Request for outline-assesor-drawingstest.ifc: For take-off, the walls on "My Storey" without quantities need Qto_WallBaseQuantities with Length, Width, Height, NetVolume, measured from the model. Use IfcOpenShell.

First a look at what the model holds.

```python
import ifcopenshell
import ifcopenshell.util.element
import ifcopenshell.util.unit

model = ifcopenshell.open("outline-assesor-drawingstest.ifc")
print(model.schema)
for unit_type in ("LENGTHUNIT", "AREAUNIT", "VOLUMEUNIT"):
    print(unit_type, ifcopenshell.util.unit.calculate_unit_scale(model, unit_type))
storey = next(s for s in model.by_type("IfcBuildingStorey") if s.Name == "My Storey")
walls = [e for e in ifcopenshell.util.element.get_decomposition(storey) if e.is_a("IfcWall")]
for e in sorted(walls, key=lambda e: e.id()):
    print(e.id(), e.is_a(), e.Name, list(ifcopenshell.util.element.get_psets(e, qtos_only=True)), sep=" | ")
```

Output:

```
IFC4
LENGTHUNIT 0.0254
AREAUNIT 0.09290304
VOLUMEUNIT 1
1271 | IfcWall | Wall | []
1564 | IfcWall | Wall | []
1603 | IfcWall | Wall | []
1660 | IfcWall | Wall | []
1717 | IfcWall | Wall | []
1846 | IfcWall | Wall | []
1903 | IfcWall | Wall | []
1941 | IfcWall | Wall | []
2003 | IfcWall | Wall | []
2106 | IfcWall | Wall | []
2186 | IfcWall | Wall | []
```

```python
import ifcopenshell
import ifcopenshell.api.pset
import ifcopenshell.geom
import ifcopenshell.util.element
import ifcopenshell.util.shape
import ifcopenshell.util.unit

model = ifcopenshell.open("outline-assesor-drawingstest.ifc")
unit_scale = ifcopenshell.util.unit.calculate_unit_scale(model)
volume_scale = ifcopenshell.util.unit.calculate_unit_scale(model, "VOLUMEUNIT")
settings = ifcopenshell.geom.settings()

storey = next(s for s in model.by_type("IfcBuildingStorey") if s.Name == "My Storey")
walls = [e for e in ifcopenshell.util.element.get_decomposition(storey) if e.is_a("IfcWall")]

for e in sorted(walls, key=lambda e: e.id()):
    if ifcopenshell.util.element.get_psets(e, qtos_only=True, should_inherit=False):
        continue
    # Geometry comes back in metres, in the element's own axes.
    shape = ifcopenshell.geom.create_shape(settings, e)
    values = {
        "Length": ifcopenshell.util.shape.get_x(shape.geometry) / unit_scale,
        "Width": ifcopenshell.util.shape.get_y(shape.geometry) / unit_scale,
        "Height": ifcopenshell.util.shape.get_z(shape.geometry) / unit_scale,
        "NetVolume": ifcopenshell.util.shape.get_volume(shape.geometry) / volume_scale,
    }
    qto = ifcopenshell.api.pset.add_qto(model, product=e, name="Qto_WallBaseQuantities")
    ifcopenshell.api.pset.edit_qto(model, qto=qto, properties=values)
    print(e.id(), {k: round(v, 3) for k, v in values.items()})

model.write("outline-assesor-drawingstest_rev.ifc")
```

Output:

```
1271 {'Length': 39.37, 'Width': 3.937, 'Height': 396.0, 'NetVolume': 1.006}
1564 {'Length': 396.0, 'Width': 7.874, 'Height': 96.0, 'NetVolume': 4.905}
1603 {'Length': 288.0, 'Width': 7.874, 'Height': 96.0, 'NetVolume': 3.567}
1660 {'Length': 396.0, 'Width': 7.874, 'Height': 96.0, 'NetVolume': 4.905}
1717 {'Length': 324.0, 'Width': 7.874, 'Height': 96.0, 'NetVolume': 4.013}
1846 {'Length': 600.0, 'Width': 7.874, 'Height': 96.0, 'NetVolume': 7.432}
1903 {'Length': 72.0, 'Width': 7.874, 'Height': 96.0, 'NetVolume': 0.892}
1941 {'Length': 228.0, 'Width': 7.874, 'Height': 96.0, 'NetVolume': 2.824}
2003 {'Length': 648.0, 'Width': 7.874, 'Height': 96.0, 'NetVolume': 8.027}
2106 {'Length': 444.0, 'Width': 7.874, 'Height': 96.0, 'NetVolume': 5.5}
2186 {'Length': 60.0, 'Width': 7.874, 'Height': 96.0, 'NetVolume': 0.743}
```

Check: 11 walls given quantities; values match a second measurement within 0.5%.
